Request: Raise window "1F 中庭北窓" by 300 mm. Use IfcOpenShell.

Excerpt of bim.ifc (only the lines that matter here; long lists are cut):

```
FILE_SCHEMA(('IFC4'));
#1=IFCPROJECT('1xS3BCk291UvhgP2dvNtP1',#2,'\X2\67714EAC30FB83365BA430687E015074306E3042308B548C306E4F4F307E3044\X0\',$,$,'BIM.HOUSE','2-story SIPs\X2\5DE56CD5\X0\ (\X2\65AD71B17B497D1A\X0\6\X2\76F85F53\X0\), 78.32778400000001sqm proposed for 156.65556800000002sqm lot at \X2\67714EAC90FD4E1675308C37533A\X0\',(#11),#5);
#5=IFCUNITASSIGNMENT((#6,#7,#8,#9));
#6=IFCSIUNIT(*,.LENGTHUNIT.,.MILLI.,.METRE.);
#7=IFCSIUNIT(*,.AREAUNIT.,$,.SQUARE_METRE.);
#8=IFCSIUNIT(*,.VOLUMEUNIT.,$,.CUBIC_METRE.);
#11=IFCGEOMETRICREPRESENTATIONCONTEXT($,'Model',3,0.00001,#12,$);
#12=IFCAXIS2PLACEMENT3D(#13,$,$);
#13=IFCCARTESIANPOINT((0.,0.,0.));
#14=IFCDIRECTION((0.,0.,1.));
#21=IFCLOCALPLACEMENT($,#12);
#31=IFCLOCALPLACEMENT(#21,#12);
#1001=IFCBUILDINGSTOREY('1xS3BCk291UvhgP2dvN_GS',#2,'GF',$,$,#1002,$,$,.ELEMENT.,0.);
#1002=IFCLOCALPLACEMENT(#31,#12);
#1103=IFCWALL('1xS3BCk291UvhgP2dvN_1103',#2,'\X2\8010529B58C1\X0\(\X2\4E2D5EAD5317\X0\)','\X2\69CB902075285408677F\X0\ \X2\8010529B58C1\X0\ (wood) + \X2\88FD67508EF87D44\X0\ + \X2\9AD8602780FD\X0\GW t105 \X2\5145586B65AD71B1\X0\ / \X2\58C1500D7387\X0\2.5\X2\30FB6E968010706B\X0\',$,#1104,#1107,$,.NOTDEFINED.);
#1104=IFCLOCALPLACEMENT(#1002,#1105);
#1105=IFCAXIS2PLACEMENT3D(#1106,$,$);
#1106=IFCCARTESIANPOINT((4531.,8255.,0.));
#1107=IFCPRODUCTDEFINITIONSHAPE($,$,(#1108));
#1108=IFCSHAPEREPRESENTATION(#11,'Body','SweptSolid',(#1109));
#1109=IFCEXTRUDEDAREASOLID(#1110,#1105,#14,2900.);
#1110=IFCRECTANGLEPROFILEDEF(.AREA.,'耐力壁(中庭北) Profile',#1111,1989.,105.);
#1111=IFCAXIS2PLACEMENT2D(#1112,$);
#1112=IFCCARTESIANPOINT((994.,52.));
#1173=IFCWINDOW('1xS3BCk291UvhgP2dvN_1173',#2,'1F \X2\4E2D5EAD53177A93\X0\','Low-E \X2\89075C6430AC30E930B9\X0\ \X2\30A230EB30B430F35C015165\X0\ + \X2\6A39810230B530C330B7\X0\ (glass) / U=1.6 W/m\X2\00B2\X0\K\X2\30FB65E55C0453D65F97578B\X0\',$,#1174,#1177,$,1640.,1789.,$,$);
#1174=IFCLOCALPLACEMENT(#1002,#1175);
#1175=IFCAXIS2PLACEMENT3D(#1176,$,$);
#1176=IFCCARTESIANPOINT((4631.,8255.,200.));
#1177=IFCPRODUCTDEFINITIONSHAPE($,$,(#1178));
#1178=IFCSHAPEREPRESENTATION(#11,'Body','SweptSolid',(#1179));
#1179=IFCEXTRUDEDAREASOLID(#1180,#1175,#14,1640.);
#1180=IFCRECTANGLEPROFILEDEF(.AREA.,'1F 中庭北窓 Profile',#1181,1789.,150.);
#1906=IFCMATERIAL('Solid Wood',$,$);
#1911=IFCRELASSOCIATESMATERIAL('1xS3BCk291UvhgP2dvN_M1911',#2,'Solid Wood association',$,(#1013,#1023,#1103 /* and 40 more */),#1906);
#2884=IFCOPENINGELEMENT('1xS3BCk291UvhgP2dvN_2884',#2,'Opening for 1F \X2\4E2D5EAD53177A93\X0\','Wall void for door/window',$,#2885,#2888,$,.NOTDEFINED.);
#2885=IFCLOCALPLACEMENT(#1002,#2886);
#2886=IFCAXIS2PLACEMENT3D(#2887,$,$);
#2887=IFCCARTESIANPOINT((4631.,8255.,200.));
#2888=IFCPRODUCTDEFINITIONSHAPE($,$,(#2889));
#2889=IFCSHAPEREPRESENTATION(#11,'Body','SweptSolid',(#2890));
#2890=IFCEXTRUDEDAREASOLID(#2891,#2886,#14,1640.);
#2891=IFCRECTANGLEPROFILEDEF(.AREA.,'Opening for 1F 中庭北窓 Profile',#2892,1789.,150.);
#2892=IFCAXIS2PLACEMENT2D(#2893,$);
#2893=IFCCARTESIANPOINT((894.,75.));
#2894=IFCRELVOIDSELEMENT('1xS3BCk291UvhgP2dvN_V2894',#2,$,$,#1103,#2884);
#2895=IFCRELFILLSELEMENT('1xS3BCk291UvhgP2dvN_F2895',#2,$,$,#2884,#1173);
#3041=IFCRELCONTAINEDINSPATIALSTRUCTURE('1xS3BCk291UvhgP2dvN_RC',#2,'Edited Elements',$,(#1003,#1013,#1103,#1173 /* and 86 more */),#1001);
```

```python
import numpy as np
import ifcopenshell
import ifcopenshell.api.geometry
import ifcopenshell.util.placement
import ifcopenshell.util.unit

model = ifcopenshell.open("bim.ifc")
unit_scale = ifcopenshell.util.unit.calculate_unit_scale(model)

window = model.by_id(1173)
opening = window.FillsVoids[0].RelatingOpeningElement
dz = 0.3 / unit_scale

shift = np.array([0.0, 0.0, dz])
# The window is not placed relative to its opening, so move both.
for product in (opening, window):
    matrix = ifcopenshell.util.placement.get_local_placement(product.ObjectPlacement)
    matrix[:3, 3] += shift
    ifcopenshell.api.geometry.edit_object_placement(model, product=product, matrix=matrix, is_si=False)

print(f"moved by {dz * unit_scale:+.3f} m")

model.write("bim_updated.ifc")
```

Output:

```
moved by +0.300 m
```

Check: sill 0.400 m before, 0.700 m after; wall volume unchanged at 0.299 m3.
